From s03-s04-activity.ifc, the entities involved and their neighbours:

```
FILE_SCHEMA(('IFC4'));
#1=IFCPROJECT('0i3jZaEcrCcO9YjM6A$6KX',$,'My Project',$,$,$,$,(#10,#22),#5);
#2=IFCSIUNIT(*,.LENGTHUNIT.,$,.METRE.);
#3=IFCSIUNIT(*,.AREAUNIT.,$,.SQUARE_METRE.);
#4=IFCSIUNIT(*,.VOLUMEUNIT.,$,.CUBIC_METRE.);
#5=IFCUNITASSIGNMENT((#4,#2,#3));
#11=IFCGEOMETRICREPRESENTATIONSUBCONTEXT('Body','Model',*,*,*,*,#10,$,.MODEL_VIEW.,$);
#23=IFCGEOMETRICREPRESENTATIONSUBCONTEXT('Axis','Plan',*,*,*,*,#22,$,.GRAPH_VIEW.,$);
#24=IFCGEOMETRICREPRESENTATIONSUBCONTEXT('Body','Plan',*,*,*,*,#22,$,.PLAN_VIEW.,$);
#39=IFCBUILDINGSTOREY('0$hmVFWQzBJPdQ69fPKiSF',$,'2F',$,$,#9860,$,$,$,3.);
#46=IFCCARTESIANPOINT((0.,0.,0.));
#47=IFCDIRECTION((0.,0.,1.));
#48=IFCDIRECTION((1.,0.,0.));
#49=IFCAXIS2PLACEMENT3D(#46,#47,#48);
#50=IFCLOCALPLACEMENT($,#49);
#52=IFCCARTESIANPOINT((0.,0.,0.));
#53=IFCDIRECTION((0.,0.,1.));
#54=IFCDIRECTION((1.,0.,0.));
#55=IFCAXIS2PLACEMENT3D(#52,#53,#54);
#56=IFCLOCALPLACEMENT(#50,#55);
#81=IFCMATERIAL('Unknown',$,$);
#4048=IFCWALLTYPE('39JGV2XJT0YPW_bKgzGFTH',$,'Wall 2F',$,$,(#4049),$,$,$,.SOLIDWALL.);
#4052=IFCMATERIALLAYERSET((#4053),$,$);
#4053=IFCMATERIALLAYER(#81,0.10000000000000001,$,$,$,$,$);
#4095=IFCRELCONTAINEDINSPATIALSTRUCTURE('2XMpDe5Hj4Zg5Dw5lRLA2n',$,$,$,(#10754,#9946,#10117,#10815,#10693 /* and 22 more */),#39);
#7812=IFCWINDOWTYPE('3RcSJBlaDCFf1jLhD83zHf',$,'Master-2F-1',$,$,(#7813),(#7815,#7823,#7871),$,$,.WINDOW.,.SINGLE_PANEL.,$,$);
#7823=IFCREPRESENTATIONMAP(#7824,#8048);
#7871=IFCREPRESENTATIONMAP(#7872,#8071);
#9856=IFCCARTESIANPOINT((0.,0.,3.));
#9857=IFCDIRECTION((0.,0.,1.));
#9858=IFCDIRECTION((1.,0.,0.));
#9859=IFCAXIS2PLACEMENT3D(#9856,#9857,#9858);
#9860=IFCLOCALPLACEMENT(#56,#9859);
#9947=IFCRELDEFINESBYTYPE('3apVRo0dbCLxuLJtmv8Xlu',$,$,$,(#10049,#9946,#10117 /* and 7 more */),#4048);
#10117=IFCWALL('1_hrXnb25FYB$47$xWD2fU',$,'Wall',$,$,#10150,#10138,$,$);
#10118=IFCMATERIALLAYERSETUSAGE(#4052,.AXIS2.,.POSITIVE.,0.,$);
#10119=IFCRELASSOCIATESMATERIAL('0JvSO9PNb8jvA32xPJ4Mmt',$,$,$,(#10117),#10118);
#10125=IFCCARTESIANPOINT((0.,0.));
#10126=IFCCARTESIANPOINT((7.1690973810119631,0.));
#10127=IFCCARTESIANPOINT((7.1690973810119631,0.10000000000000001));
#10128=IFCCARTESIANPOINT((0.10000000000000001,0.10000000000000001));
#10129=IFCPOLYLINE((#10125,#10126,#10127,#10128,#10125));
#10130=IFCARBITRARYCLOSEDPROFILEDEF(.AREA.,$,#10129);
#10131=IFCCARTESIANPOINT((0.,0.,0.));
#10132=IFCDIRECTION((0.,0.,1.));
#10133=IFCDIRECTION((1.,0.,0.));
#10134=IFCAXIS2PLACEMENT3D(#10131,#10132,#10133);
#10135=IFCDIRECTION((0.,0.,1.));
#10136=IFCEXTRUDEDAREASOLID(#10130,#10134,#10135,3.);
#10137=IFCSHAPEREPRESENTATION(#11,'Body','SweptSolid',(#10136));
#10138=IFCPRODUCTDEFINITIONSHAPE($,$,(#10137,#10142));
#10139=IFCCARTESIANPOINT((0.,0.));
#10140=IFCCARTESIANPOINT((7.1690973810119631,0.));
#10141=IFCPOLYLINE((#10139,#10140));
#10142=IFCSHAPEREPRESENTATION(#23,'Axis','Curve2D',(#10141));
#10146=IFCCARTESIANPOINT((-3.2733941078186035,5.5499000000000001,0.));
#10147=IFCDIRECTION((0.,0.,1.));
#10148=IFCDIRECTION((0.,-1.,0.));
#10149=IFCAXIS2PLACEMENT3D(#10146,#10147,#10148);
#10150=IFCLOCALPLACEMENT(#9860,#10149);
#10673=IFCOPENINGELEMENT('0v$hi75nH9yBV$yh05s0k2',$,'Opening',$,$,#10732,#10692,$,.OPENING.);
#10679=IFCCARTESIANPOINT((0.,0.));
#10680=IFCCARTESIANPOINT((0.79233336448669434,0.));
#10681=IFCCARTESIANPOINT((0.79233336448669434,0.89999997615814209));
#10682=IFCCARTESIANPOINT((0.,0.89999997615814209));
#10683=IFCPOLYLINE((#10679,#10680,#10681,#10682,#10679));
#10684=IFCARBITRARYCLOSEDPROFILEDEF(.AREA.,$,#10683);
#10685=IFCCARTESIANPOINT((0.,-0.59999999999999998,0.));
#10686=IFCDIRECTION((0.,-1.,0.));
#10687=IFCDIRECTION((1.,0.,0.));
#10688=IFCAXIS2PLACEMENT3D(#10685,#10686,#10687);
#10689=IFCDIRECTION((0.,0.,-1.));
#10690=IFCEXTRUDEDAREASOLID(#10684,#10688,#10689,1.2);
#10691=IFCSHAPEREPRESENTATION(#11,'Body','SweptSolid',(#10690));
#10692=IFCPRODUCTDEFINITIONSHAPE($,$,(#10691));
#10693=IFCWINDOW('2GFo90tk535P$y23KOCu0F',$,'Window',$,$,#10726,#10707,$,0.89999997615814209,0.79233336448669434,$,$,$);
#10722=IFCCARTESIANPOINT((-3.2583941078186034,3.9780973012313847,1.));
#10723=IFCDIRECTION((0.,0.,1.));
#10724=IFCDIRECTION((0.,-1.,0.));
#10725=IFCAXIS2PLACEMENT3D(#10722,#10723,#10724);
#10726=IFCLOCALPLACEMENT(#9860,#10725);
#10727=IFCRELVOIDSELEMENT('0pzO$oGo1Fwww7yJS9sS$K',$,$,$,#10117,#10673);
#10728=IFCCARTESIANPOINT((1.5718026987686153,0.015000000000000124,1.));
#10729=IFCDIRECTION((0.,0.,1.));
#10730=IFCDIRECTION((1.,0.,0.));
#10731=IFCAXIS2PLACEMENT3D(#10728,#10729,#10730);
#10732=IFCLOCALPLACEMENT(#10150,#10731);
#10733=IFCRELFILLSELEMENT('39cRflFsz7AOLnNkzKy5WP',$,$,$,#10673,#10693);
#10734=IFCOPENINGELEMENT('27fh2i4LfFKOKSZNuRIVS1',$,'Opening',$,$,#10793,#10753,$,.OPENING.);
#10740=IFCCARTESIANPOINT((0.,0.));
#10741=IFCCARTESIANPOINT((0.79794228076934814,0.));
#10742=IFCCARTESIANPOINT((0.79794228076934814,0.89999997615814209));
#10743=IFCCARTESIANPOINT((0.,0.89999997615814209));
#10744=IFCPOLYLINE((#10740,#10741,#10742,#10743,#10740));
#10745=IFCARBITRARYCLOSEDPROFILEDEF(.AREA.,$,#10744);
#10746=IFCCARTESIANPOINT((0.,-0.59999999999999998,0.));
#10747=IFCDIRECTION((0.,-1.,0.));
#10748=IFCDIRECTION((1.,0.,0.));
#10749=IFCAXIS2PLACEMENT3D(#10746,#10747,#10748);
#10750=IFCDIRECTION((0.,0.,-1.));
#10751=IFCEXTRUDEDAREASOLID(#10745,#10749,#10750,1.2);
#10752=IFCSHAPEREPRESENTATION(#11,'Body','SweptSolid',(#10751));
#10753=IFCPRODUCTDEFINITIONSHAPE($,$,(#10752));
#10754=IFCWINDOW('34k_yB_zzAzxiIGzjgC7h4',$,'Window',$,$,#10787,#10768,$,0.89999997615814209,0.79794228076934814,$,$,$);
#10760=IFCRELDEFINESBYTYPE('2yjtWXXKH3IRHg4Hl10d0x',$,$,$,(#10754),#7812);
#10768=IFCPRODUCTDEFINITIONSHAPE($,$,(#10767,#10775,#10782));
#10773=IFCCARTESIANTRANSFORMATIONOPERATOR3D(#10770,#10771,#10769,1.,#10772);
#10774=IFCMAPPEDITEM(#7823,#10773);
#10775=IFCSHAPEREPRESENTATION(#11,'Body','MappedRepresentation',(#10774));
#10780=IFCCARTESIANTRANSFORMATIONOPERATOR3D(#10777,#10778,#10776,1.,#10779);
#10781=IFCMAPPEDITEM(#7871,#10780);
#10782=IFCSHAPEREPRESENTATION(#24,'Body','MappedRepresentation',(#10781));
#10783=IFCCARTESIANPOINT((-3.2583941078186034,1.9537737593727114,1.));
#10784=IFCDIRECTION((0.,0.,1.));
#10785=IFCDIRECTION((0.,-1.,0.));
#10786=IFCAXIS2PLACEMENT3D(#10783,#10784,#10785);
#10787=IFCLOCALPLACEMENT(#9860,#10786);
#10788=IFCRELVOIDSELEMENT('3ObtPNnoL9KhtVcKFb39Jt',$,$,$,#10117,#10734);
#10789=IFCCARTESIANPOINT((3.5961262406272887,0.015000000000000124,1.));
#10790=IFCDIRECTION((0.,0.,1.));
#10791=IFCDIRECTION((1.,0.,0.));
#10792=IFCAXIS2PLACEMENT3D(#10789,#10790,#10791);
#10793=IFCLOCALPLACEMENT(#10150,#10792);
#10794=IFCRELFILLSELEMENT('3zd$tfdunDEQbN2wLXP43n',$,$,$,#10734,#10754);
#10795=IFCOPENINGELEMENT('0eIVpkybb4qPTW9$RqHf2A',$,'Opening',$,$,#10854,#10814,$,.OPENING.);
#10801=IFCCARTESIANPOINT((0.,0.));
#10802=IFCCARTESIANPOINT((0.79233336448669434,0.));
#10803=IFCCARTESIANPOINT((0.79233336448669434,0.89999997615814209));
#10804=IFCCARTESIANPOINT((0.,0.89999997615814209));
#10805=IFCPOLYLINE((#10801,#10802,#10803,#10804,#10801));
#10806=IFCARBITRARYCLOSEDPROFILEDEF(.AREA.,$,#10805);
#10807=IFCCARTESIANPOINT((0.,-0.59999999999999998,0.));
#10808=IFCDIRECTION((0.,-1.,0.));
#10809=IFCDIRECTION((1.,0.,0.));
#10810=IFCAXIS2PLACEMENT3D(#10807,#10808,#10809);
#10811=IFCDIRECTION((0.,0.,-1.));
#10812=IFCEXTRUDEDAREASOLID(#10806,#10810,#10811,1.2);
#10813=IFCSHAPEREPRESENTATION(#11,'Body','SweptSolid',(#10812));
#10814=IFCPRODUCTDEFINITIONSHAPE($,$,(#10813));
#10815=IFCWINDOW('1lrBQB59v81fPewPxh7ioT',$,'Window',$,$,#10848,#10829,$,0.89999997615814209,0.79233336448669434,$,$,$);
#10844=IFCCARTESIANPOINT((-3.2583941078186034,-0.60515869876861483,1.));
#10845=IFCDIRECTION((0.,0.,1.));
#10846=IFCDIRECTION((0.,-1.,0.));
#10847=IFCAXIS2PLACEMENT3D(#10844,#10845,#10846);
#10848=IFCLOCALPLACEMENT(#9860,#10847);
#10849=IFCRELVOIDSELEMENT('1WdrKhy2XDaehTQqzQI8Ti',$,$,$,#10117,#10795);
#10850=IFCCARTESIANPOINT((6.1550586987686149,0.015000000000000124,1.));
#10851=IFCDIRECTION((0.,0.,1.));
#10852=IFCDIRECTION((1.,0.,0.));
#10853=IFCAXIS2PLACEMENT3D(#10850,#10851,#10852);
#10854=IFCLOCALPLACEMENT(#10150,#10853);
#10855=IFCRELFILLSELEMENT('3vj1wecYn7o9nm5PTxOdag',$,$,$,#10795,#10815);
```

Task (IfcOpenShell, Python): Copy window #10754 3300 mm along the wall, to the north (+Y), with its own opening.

```python
import ifcopenshell
import ifcopenshell.api.feature
import ifcopenshell.api.geometry
import ifcopenshell.api.root
import ifcopenshell.geom
import ifcopenshell.util.element
import ifcopenshell.util.placement
import ifcopenshell.util.shape
import ifcopenshell.util.unit

model = ifcopenshell.open("s03-s04-activity.ifc")
unit_scale = ifcopenshell.util.unit.calculate_unit_scale(model)
settings = ifcopenshell.geom.settings()


def volume(element):
    """Net volume in cubic metres, openings subtracted."""
    shape = ifcopenshell.geom.create_shape(settings, element)
    return ifcopenshell.util.shape.get_volume(shape.geometry)


window = model.by_id(10754)
opening = window.FillsVoids[0].RelatingOpeningElement
wall = opening.VoidsElements[0].RelatingBuildingElement
before = volume(wall)
shift = ifcopenshell.util.placement.get_local_placement(wall.ObjectPlacement)[:3, 0] * -3.3 / unit_scale

# copy_class copies the void relationship, type, container and properties, but no geometry.
new_opening = ifcopenshell.api.root.copy_class(model, product=opening)
new_opening.Representation = ifcopenshell.util.element.copy_deep(
    model, opening.Representation, exclude=["IfcGeometricRepresentationContext", "IfcRepresentationMap"]
)
new_window = ifcopenshell.api.root.copy_class(model, product=window)
new_window.Representation = ifcopenshell.util.element.copy_deep(
    model, window.Representation, exclude=["IfcGeometricRepresentationContext", "IfcRepresentationMap"]
)
ifcopenshell.api.feature.add_filling(model, opening=new_opening, element=new_window)

for old, new in ((opening, new_opening), (window, new_window)):
    matrix = ifcopenshell.util.placement.get_local_placement(old.ObjectPlacement)
    matrix[:3, 3] += shift
    ifcopenshell.api.geometry.edit_object_placement(model, product=new, matrix=matrix, is_si=False)

after = volume(wall)

print(f"wall volume {before:.3f} -> {after:.3f} m3")

model.write("s03-s04-activity_edited.ifc")
```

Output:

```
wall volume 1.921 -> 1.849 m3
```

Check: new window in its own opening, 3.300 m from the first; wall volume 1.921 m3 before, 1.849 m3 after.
